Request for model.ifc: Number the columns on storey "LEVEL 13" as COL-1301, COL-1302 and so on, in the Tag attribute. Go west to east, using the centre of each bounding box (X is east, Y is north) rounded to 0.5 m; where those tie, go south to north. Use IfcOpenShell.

First a look at what the model holds.

```python
import ifcopenshell
import ifcopenshell.util.element
import ifcopenshell.util.placement

model = ifcopenshell.open("model.ifc")
print(model.schema)
storey = next(s for s in model.by_type("IfcBuildingStorey") if s.Name == "LEVEL 13")
columns = [e for e in ifcopenshell.util.element.get_decomposition(storey) if e.is_a("IfcColumn")]
for e in sorted(columns, key=lambda e: e.id()):
    origin = ifcopenshell.util.placement.get_local_placement(e.ObjectPlacement)[:3, 3]
    print(e.id(), e.Tag, e.Name, origin.round(2) + 0.0, sep=" | ")
```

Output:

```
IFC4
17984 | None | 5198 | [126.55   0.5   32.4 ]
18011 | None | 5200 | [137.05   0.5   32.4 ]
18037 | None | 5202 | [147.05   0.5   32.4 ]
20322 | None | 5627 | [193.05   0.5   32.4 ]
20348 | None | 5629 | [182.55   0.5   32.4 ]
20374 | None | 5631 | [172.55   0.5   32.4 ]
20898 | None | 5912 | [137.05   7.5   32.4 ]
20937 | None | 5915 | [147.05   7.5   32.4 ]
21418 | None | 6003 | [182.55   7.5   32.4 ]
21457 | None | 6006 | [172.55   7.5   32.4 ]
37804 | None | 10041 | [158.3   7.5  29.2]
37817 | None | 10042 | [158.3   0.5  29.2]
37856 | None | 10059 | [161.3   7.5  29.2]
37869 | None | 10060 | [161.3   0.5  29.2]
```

```python
import ifcopenshell
import ifcopenshell.geom
import ifcopenshell.util.element
import ifcopenshell.util.shape

model = ifcopenshell.open("model.ifc")
settings = ifcopenshell.geom.settings()
settings.set("use-world-coords", True)


def centre(element):
    shape = ifcopenshell.geom.create_shape(settings, element)
    return ifcopenshell.util.shape.get_bbox_centroid(shape.geometry)


storey = next(s for s in model.by_type("IfcBuildingStorey") if s.Name == "LEVEL 13")
columns = [e for e in ifcopenshell.util.element.get_decomposition(storey) if e.is_a("IfcColumn")]

# Insertion points can sit at a corner or the storey origin, so sort by the geometry (in metres).
centres = {e: centre(e) for e in columns}
columns.sort(key=lambda e: (round(centres[e][0] / 0.5), centres[e][1]))

for i, e in enumerate(columns, start=1):
    number = f"COL-13{i:02d}"
    e.Tag = number
    print(e.id(), number)

model.write("model_updated.ifc")
```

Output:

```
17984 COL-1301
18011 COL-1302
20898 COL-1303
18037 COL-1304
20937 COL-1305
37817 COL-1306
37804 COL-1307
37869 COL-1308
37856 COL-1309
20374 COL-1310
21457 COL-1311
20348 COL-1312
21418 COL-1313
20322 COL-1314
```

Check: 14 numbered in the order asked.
